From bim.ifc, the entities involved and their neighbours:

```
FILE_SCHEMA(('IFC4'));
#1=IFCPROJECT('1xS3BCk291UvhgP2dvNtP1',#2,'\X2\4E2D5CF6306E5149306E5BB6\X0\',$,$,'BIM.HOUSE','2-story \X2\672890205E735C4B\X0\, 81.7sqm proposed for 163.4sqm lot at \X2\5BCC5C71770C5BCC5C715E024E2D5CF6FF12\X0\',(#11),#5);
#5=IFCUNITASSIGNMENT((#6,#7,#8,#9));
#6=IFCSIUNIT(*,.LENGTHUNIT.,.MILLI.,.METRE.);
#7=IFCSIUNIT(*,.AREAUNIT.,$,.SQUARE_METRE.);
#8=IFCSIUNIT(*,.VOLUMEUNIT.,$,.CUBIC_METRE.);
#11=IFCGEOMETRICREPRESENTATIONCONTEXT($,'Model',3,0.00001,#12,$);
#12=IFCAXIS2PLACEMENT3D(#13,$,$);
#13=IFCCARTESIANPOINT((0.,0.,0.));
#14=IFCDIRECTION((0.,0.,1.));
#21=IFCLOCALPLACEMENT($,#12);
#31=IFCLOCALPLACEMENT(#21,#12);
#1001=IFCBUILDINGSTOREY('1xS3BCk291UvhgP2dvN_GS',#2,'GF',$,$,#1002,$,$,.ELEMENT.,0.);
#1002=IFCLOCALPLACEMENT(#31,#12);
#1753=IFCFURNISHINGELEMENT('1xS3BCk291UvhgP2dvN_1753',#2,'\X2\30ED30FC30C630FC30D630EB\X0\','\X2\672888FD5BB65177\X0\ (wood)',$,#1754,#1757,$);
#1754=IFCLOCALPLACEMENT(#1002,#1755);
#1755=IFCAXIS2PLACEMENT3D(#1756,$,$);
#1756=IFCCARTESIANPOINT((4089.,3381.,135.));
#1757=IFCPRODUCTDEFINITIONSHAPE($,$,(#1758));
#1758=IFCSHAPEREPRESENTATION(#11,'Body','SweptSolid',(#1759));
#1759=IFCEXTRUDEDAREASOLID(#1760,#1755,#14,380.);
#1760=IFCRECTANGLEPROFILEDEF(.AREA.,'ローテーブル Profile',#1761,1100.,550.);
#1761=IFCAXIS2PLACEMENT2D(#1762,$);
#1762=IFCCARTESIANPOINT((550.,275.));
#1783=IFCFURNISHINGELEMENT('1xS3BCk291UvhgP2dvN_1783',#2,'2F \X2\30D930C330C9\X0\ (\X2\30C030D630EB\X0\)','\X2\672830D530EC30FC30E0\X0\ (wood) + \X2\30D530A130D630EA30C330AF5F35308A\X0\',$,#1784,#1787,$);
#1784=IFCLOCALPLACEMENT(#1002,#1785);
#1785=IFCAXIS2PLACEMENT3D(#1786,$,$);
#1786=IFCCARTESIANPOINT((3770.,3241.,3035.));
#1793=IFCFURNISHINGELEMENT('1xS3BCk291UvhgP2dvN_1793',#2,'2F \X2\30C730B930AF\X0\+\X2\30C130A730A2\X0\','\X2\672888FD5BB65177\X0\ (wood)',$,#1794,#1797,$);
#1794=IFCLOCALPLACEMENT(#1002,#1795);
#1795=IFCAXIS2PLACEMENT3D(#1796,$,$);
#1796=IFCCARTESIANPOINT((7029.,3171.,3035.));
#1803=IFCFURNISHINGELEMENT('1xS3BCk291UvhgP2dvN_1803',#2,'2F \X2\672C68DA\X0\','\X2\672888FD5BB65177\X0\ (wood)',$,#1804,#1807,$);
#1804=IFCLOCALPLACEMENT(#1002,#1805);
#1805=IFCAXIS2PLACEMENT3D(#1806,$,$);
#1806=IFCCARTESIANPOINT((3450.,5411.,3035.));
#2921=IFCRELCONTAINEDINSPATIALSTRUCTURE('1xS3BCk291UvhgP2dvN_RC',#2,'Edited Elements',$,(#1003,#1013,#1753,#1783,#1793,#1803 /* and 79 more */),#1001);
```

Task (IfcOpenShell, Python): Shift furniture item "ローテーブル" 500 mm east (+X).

```python
import ifcopenshell
import ifcopenshell.api.geometry
import ifcopenshell.util.placement
import ifcopenshell.util.unit

model = ifcopenshell.open("bim.ifc")
unit_scale = ifcopenshell.util.unit.calculate_unit_scale(model)

item = model.by_guid("1xS3BCk291UvhgP2dvN_1753")
matrix = ifcopenshell.util.placement.get_local_placement(item.ObjectPlacement)
matrix[0, 3] += 0.5 / unit_scale
ifcopenshell.api.geometry.edit_object_placement(model, product=item, matrix=matrix, is_si=False)

print(ifcopenshell.util.placement.get_local_placement(item.ObjectPlacement).round(3) + 0.0)

model.write("bim_edited.ifc")
```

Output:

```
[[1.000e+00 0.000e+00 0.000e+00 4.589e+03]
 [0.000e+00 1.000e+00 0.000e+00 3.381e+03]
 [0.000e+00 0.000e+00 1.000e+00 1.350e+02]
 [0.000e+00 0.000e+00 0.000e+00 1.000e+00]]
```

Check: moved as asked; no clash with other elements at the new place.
